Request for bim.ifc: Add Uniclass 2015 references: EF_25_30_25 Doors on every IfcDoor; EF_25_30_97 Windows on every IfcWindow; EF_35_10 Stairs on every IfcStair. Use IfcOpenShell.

First a look at what the model holds.

```python
import ifcopenshell

model = ifcopenshell.open("bim.ifc")
print(model.schema)
print("classifications:", [c.Name for c in model.by_type("IfcClassification")])
for ifc_class in ("IfcDoor", "IfcRoof", "IfcStair", "IfcWall", "IfcWindow"):
    print(ifc_class, len(model.by_type(ifc_class)))
```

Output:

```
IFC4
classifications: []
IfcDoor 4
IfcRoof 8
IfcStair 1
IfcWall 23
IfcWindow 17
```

```python
import ifcopenshell
import ifcopenshell.api.classification

model = ifcopenshell.open("bim.ifc")

system = ifcopenshell.api.classification.add_classification(model, classification="Uniclass 2015")

codes = {
    "IfcDoor": ("EF_25_30_25", "Doors"),
    "IfcWindow": ("EF_25_30_97", "Windows"),
    "IfcStair": ("EF_35_10", "Stairs"),
}
for ifc_class, (code, name) in codes.items():
    products = model.by_type(ifc_class)
    ifcopenshell.api.classification.add_reference(
        model, products=products, classification=system, identification=code, name=name
    )
    print(code, len(products))

model.write("bim_edited.ifc")
```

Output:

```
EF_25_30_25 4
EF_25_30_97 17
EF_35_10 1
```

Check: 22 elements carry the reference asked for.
